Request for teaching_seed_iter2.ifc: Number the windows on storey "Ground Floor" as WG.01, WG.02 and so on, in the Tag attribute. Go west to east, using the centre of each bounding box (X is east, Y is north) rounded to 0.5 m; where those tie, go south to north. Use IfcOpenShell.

First a look at what the model holds.

```python
import ifcopenshell
import ifcopenshell.util.element
import ifcopenshell.util.placement

model = ifcopenshell.open("teaching_seed_iter2.ifc")
print(model.schema)
storey = next(s for s in model.by_type("IfcBuildingStorey") if s.Name == "Ground Floor")
windows = [e for e in ifcopenshell.util.element.get_decomposition(storey) if e.is_a("IfcWindow")]
for e in sorted(windows, key=lambda e: e.id()):
    origin = ifcopenshell.util.placement.get_local_placement(e.ObjectPlacement)[:3, 3]
    print(e.id(), e.Tag, e.Name, origin.round(2) + 0.0, sep=" | ")
```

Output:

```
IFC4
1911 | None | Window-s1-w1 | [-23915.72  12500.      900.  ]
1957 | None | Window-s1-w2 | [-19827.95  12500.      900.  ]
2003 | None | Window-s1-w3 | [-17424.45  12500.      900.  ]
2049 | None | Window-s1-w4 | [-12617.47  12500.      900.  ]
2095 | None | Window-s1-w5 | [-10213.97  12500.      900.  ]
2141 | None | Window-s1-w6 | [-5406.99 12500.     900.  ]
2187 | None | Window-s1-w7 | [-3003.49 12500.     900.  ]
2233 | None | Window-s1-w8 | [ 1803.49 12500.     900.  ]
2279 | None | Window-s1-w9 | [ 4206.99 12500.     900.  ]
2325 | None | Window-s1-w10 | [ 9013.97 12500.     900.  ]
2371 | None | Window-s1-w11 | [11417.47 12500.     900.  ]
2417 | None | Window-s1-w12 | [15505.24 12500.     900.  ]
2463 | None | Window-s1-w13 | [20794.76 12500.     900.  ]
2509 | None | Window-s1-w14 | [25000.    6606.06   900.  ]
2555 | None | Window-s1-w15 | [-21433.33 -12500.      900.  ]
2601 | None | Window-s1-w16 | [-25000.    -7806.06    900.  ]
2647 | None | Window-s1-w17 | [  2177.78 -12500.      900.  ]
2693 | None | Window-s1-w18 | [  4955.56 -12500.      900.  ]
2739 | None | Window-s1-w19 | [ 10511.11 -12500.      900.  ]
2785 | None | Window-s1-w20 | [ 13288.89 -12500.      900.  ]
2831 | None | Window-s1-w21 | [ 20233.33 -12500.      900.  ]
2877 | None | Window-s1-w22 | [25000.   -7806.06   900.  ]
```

```python
import ifcopenshell
import ifcopenshell.geom
import ifcopenshell.util.element
import ifcopenshell.util.shape

model = ifcopenshell.open("teaching_seed_iter2.ifc")
settings = ifcopenshell.geom.settings()
settings.set("use-world-coords", True)


def centre(element):
    shape = ifcopenshell.geom.create_shape(settings, element)
    return ifcopenshell.util.shape.get_bbox_centroid(shape.geometry)


storey = next(s for s in model.by_type("IfcBuildingStorey") if s.Name == "Ground Floor")
windows = [e for e in ifcopenshell.util.element.get_decomposition(storey) if e.is_a("IfcWindow")]

# Insertion points can sit at a corner or the storey origin, so sort by the geometry (in metres).
centres = {e: centre(e) for e in windows}
windows.sort(key=lambda e: (round(centres[e][0] / 0.5), centres[e][1]))

for i, e in enumerate(windows, start=1):
    number = f"WG.{i:02d}"
    e.Tag = number
    print(e.id(), number)

model.write("teaching_seed_iter2_v2.ifc")
```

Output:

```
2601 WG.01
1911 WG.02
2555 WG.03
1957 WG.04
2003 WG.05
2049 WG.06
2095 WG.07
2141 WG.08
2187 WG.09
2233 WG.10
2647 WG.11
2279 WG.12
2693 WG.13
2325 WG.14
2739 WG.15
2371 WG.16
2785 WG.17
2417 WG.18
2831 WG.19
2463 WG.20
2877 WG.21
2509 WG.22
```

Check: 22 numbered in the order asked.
